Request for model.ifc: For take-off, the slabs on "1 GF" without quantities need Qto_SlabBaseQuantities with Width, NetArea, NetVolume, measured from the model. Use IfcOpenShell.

First a look at what the model holds.

```python
import ifcopenshell
import ifcopenshell.util.element
import ifcopenshell.util.unit

model = ifcopenshell.open("model.ifc")
print(model.schema)
for unit_type in ("LENGTHUNIT", "AREAUNIT", "VOLUMEUNIT"):
    print(unit_type, ifcopenshell.util.unit.calculate_unit_scale(model, unit_type))
storey = next(s for s in model.by_type("IfcBuildingStorey") if s.Name == "1 GF")
slabs = [e for e in ifcopenshell.util.element.get_decomposition(storey) if e.is_a("IfcSlab")]
for e in sorted(slabs, key=lambda e: e.id()):
    print(e.id(), e.is_a(), e.Name, list(ifcopenshell.util.element.get_psets(e, qtos_only=True)), sep=" | ")
```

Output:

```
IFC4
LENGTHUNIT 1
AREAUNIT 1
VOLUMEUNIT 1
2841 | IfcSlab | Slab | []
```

```python
import ifcopenshell
import ifcopenshell.api.pset
import ifcopenshell.geom
import ifcopenshell.util.element
import ifcopenshell.util.shape
import ifcopenshell.util.unit

model = ifcopenshell.open("model.ifc")
unit_scale = ifcopenshell.util.unit.calculate_unit_scale(model)
area_scale = ifcopenshell.util.unit.calculate_unit_scale(model, "AREAUNIT")
volume_scale = ifcopenshell.util.unit.calculate_unit_scale(model, "VOLUMEUNIT")
settings = ifcopenshell.geom.settings()

storey = next(s for s in model.by_type("IfcBuildingStorey") if s.Name == "1 GF")
slabs = [e for e in ifcopenshell.util.element.get_decomposition(storey) if e.is_a("IfcSlab")]

for e in sorted(slabs, key=lambda e: e.id()):
    if ifcopenshell.util.element.get_psets(e, qtos_only=True, should_inherit=False):
        continue
    # Geometry comes back in metres, in the element's own axes.
    shape = ifcopenshell.geom.create_shape(settings, e)
    values = {
        "Width": ifcopenshell.util.shape.get_z(shape.geometry) / unit_scale,
        "NetArea": ifcopenshell.util.shape.get_footprint_area(shape.geometry) / area_scale,
        "NetVolume": ifcopenshell.util.shape.get_volume(shape.geometry) / volume_scale,
    }
    qto = ifcopenshell.api.pset.add_qto(model, product=e, name="Qto_SlabBaseQuantities")
    ifcopenshell.api.pset.edit_qto(model, qto=qto, properties=values)
    print(e.id(), {k: round(v, 3) for k, v in values.items()})

model.write("model_rev.ifc")
```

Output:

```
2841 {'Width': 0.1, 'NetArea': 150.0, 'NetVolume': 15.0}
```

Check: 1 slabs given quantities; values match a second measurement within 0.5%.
